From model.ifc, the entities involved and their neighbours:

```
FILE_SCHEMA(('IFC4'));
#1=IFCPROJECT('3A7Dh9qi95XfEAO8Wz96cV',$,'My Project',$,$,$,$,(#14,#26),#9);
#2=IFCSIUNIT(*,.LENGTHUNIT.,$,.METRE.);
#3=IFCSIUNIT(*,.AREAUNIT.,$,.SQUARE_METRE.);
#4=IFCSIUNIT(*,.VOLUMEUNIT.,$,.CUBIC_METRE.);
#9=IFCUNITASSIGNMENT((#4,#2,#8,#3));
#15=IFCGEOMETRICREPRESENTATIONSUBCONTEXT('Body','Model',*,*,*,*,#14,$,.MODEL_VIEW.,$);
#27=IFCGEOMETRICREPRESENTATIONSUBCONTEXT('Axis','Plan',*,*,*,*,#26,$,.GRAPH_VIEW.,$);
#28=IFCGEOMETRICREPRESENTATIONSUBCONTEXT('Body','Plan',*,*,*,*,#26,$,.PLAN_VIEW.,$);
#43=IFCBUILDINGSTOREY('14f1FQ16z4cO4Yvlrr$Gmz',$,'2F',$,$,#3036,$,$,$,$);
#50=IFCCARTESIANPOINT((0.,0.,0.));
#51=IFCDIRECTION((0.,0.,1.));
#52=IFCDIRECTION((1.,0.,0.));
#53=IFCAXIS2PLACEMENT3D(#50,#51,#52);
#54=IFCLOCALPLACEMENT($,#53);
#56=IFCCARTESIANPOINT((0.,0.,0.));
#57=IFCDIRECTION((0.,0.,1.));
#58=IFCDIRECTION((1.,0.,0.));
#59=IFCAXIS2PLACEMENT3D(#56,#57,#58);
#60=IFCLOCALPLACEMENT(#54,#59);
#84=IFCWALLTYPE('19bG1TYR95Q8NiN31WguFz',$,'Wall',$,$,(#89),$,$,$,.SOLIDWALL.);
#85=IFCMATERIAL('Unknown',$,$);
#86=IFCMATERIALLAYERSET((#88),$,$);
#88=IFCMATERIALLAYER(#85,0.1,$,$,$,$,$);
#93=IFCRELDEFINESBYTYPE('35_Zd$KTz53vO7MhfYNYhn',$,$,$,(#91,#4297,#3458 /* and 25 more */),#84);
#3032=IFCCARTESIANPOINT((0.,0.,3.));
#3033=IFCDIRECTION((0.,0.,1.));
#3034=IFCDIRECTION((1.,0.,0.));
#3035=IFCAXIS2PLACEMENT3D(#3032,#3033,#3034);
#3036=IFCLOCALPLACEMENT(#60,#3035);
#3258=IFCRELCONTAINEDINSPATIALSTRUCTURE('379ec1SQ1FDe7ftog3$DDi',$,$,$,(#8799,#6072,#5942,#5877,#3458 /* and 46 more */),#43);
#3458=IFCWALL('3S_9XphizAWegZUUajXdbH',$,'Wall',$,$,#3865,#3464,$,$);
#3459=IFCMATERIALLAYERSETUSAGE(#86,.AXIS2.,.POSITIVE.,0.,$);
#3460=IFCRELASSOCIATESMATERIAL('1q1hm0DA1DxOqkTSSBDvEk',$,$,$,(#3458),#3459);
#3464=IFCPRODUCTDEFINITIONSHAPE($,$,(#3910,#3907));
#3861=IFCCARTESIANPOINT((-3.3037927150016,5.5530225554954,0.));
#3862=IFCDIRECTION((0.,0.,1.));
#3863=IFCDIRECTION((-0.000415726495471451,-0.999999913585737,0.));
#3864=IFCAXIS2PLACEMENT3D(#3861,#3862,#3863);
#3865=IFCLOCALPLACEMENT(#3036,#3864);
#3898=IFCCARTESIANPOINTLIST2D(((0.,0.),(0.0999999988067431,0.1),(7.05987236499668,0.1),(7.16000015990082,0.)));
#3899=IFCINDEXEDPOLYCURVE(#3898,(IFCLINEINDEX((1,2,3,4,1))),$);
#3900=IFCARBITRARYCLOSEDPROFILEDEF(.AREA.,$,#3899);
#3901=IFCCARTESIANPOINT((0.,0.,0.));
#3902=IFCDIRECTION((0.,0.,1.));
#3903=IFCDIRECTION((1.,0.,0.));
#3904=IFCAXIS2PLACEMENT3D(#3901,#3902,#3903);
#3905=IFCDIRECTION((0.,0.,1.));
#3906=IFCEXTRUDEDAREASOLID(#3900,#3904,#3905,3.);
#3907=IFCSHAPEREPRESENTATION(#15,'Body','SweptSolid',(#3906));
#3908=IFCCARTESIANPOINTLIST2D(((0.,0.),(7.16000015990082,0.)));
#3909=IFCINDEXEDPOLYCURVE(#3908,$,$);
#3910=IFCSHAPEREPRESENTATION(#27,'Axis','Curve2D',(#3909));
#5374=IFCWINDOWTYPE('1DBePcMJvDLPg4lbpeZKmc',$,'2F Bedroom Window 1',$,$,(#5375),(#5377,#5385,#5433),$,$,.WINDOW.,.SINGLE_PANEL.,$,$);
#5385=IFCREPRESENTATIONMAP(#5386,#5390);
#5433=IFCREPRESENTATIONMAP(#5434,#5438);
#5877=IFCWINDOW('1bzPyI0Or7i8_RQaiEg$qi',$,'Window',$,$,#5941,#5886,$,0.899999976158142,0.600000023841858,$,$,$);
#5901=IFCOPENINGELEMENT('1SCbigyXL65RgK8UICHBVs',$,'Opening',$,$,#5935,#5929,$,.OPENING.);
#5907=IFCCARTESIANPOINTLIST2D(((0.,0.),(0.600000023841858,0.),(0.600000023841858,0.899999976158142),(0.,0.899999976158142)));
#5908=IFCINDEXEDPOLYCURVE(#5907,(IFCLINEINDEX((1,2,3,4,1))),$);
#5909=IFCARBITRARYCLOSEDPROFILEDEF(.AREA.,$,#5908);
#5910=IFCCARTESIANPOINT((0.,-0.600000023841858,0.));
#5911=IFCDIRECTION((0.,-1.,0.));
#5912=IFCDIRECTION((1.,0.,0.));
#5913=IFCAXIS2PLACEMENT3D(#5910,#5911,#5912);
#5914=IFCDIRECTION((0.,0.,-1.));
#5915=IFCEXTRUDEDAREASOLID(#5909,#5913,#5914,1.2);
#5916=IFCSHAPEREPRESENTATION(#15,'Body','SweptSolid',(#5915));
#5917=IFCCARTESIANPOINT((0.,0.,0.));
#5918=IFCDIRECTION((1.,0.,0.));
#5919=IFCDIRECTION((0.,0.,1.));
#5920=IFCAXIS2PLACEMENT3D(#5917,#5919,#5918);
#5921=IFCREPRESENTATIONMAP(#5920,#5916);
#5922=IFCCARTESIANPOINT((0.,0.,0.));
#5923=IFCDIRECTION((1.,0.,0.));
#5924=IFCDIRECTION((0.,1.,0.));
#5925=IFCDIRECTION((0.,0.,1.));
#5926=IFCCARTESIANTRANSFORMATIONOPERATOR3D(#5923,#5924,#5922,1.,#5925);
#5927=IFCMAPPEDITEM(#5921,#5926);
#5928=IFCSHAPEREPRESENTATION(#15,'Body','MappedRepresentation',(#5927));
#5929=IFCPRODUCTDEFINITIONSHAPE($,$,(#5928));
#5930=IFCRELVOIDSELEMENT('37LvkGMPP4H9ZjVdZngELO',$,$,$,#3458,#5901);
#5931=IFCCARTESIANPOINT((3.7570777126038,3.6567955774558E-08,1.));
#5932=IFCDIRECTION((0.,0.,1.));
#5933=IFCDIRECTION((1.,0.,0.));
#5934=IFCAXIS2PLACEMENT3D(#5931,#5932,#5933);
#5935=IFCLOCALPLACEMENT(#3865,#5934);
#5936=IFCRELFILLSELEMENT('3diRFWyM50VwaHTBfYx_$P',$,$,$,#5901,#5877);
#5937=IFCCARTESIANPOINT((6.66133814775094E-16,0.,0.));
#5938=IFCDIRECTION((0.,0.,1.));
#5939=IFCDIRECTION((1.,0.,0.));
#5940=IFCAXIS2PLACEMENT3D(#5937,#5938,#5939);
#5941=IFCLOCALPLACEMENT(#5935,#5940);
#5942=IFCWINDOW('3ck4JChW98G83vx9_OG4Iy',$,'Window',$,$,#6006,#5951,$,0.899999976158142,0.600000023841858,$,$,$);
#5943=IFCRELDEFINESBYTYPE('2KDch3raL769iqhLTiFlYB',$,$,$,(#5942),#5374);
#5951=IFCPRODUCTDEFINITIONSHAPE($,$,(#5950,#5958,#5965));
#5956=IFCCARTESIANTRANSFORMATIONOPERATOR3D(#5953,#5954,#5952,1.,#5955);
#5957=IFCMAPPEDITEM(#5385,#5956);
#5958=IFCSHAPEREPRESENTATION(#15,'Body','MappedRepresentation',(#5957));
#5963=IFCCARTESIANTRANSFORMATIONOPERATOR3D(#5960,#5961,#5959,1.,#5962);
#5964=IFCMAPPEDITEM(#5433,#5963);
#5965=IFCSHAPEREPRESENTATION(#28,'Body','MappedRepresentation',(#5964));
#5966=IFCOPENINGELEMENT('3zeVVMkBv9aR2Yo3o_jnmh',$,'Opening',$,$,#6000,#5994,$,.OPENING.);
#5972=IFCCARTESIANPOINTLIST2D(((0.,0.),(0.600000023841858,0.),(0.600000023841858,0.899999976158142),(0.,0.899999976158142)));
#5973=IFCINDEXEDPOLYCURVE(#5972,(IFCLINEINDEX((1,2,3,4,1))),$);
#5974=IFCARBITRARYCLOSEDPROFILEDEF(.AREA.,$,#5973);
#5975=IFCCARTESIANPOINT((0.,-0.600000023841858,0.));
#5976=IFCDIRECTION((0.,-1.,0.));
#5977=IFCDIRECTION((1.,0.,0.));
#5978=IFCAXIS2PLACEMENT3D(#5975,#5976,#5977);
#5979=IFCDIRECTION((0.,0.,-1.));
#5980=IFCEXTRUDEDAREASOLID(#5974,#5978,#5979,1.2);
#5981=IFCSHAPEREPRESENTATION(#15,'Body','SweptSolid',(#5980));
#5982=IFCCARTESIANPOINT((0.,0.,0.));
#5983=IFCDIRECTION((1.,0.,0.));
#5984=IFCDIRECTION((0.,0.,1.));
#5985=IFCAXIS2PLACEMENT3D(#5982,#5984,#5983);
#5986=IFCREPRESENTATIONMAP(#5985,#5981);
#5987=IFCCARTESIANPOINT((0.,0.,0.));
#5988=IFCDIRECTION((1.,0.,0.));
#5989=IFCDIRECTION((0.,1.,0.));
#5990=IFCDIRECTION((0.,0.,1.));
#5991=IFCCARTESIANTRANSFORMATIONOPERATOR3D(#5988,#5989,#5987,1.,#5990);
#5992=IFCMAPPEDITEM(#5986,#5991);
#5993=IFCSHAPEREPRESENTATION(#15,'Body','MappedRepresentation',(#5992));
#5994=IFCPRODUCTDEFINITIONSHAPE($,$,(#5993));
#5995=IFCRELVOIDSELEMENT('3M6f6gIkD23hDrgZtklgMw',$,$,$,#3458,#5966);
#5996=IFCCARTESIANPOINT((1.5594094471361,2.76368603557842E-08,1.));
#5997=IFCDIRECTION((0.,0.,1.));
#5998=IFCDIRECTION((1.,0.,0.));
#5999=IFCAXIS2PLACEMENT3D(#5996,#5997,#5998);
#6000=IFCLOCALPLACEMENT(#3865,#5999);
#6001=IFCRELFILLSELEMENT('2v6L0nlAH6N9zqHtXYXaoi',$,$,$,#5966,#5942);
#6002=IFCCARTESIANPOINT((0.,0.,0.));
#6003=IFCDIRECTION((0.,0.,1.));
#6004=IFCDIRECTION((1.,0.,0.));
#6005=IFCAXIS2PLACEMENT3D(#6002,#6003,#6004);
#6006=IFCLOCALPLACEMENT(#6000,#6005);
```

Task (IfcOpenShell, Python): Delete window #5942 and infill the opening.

```python
import ifcopenshell
import ifcopenshell.api.feature
import ifcopenshell.api.root
import ifcopenshell.geom
import ifcopenshell.util.shape

model = ifcopenshell.open("model.ifc")
settings = ifcopenshell.geom.settings()


def volume(element):
    """Net volume in cubic metres, openings subtracted."""
    shape = ifcopenshell.geom.create_shape(settings, element)
    return ifcopenshell.util.shape.get_volume(shape.geometry)


window = model.by_guid("3ck4JChW98G83vx9_OG4Iy")
opening = window.FillsVoids[0].RelatingOpeningElement
wall = opening.VoidsElements[0].RelatingBuildingElement
before = volume(wall)

ifcopenshell.api.root.remove_product(model, product=window)
ifcopenshell.api.feature.remove_feature(model, feature=opening)

after = volume(wall)

print(f"wall volume {before:.3f} -> {after:.3f} m3")

model.write("model_v2.ifc")
```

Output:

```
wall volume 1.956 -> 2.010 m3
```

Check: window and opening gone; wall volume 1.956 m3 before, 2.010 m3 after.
